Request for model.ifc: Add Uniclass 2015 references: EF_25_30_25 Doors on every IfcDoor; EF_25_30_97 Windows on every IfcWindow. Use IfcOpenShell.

First a look at what the model holds.

```python
import ifcopenshell

model = ifcopenshell.open("model.ifc")
print(model.schema)
print("classifications:", [c.Name for c in model.by_type("IfcClassification")])
for ifc_class in ("IfcDoor", "IfcRoof", "IfcStair", "IfcWall", "IfcWindow"):
    print(ifc_class, len(model.by_type(ifc_class)))
```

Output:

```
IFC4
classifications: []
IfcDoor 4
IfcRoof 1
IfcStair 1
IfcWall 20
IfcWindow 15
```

```python
import ifcopenshell
import ifcopenshell.api.classification

model = ifcopenshell.open("model.ifc")

system = ifcopenshell.api.classification.add_classification(model, classification="Uniclass 2015")

codes = {
    "IfcDoor": ("EF_25_30_25", "Doors"),
    "IfcWindow": ("EF_25_30_97", "Windows"),
}
for ifc_class, (code, name) in codes.items():
    products = model.by_type(ifc_class)
    ifcopenshell.api.classification.add_reference(
        model, products=products, classification=system, identification=code, name=name
    )
    print(code, len(products))

model.write("model-out.ifc")
```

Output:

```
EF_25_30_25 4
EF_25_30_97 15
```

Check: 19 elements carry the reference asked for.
